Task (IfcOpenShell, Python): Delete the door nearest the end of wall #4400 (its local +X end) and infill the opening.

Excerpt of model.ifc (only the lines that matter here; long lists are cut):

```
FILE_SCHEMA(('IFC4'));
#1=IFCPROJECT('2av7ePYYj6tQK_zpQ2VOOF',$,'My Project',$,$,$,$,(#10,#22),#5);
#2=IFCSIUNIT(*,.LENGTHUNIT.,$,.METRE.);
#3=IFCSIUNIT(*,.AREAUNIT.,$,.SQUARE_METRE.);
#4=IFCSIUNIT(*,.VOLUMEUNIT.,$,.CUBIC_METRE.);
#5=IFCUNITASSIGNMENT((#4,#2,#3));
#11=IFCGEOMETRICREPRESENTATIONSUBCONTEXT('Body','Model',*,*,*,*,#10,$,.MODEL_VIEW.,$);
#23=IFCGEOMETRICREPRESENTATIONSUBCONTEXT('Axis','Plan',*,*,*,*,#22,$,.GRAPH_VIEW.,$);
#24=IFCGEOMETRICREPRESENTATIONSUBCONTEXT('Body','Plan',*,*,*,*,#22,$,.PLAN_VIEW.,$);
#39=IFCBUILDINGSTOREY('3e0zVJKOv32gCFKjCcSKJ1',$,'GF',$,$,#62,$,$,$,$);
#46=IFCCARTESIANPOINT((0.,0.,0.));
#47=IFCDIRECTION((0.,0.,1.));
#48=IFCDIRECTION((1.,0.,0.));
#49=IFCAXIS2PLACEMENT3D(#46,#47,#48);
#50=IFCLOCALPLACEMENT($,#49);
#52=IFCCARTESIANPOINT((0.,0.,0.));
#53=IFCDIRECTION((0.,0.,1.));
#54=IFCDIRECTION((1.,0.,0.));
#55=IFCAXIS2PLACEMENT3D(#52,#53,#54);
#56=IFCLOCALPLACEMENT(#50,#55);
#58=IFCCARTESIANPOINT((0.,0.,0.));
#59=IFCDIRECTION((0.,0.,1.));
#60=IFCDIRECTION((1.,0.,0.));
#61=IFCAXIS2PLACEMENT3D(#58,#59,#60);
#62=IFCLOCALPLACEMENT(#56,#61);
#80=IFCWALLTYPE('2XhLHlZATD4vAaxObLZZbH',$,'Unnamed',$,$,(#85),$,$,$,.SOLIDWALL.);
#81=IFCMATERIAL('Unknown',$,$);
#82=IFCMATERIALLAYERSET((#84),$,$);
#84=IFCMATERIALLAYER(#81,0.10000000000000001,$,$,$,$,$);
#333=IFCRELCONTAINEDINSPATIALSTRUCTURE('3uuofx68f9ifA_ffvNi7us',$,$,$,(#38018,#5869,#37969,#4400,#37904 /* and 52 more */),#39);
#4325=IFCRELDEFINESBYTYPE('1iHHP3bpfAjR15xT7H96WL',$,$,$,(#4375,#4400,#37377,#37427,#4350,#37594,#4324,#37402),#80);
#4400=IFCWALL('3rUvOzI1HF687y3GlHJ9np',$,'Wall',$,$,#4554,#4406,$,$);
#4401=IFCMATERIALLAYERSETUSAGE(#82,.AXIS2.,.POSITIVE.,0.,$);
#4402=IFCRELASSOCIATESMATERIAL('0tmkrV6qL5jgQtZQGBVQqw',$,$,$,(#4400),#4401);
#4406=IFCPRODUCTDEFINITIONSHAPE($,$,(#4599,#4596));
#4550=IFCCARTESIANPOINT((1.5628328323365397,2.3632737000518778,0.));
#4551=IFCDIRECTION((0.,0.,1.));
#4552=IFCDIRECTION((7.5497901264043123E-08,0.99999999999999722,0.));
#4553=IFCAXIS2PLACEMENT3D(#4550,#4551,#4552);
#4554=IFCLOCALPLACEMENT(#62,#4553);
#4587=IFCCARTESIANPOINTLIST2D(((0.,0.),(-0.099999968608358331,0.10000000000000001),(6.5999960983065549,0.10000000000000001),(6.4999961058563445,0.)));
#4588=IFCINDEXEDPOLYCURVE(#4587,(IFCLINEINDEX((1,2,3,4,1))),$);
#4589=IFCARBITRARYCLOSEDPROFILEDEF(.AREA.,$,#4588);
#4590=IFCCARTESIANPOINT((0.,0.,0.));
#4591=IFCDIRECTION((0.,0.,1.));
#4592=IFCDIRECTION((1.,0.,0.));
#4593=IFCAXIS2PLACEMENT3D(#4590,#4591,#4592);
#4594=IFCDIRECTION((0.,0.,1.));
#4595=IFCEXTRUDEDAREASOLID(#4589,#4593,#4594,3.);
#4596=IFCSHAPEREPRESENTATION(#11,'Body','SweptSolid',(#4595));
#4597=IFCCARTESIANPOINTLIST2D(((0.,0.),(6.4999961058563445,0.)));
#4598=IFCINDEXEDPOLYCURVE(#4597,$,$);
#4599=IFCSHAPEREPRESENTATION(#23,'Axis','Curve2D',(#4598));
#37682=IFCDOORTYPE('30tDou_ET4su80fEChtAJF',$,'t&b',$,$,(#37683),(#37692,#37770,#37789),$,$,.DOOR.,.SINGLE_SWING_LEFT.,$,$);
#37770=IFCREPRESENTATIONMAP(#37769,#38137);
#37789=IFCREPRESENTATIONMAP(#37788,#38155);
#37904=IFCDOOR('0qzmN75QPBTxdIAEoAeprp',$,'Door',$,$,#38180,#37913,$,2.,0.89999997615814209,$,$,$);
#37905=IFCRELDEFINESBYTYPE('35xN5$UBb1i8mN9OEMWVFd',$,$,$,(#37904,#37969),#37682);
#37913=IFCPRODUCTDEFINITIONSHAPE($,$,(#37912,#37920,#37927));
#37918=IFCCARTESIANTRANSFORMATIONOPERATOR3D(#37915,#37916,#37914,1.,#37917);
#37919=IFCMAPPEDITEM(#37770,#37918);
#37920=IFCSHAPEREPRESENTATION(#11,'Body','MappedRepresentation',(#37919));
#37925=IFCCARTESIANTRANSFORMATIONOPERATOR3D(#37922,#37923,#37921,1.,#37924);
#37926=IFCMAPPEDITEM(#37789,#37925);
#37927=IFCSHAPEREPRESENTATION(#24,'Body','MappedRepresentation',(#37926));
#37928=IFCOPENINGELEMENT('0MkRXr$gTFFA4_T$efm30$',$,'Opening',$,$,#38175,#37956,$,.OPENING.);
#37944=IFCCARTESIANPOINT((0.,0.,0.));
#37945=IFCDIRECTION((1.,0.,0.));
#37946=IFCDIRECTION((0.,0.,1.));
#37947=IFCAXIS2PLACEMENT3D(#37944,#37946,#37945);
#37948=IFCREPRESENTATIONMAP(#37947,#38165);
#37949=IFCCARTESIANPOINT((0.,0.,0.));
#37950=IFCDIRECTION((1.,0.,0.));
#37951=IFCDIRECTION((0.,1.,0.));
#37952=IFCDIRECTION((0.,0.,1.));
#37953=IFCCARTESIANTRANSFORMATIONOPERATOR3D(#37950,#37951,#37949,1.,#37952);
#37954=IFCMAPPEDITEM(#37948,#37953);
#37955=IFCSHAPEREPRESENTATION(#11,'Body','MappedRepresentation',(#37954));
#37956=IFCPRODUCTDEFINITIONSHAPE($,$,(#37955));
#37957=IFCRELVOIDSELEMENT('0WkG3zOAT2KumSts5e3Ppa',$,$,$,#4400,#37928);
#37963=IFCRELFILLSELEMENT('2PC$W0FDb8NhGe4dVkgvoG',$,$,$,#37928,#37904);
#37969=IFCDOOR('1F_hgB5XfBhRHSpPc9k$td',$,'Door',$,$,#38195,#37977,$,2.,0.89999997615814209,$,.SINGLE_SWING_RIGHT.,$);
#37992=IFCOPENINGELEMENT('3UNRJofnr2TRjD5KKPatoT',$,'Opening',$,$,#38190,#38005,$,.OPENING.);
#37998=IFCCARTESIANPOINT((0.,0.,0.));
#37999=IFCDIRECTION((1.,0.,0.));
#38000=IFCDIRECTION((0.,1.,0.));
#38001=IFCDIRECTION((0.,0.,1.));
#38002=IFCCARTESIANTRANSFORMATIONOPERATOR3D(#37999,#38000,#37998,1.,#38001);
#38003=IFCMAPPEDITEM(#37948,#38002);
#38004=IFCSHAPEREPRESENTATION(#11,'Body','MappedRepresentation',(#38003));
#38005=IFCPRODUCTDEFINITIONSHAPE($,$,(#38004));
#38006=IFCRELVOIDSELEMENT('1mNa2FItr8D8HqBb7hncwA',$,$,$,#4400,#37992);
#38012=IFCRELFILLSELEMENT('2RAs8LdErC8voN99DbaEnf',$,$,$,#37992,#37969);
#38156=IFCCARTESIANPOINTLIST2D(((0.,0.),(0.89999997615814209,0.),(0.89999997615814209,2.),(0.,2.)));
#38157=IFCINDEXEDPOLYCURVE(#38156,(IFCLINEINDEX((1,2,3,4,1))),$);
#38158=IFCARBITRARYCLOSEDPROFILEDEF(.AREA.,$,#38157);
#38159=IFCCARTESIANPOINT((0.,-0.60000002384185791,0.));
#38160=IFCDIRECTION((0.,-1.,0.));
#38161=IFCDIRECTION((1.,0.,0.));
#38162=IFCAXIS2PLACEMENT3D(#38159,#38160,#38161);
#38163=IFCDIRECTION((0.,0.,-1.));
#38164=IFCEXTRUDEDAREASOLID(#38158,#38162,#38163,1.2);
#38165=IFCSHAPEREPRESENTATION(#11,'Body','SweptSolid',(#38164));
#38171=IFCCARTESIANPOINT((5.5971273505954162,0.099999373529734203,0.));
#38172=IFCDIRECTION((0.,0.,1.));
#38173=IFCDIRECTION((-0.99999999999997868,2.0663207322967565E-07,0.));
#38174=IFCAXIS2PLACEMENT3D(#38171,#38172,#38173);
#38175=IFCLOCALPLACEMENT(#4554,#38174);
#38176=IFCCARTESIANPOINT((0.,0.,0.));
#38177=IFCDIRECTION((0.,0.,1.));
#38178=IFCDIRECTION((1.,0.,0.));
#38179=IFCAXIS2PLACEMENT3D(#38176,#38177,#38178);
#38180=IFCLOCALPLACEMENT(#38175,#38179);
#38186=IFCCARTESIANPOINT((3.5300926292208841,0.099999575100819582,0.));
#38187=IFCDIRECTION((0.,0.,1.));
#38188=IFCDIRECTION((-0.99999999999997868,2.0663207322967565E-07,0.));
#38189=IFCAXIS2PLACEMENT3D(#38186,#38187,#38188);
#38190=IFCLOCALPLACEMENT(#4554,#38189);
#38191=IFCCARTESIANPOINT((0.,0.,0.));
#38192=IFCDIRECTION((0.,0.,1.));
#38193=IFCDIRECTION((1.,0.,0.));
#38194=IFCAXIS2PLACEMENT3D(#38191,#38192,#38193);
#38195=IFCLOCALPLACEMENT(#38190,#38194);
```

```python
import ifcopenshell
import ifcopenshell.api.feature
import ifcopenshell.api.root
import ifcopenshell.geom
import ifcopenshell.util.shape

model = ifcopenshell.open("model.ifc")
settings = ifcopenshell.geom.settings()


def volume(element):
    """Net volume in cubic metres, openings subtracted."""
    shape = ifcopenshell.geom.create_shape(settings, element)
    return ifcopenshell.util.shape.get_volume(shape.geometry)


door = model.by_id(37904)
opening = door.FillsVoids[0].RelatingOpeningElement
wall = opening.VoidsElements[0].RelatingBuildingElement
before = volume(wall)

ifcopenshell.api.root.remove_product(model, product=door)
ifcopenshell.api.feature.remove_feature(model, feature=opening)

after = volume(wall)

print(f"wall volume {before:.3f} -> {after:.3f} m3")

model.write("model_v2.ifc")
```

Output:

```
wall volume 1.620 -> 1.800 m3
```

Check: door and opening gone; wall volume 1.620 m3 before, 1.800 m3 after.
